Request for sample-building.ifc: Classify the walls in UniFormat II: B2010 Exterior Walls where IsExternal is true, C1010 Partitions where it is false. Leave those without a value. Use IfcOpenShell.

First a look at what the model holds.

```python
import ifcopenshell
import ifcopenshell.util.element

model = ifcopenshell.open("sample-building.ifc")
print(model.schema)
print("classifications:", [c.Name for c in model.by_type("IfcClassification")])
values = [ifcopenshell.util.element.get_pset(e, "Pset_WallCommon", "IsExternal") for e in model.by_type("IfcWall")]
for value in (True, False, None):
    print("IsExternal", value, values.count(value))
```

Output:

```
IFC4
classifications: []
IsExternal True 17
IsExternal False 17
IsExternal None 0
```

```python
import ifcopenshell
import ifcopenshell.api.classification
import ifcopenshell.util.element

model = ifcopenshell.open("sample-building.ifc")

system = ifcopenshell.api.classification.add_classification(model, classification="UniFormat II")

walls = model.by_type("IfcWall")
external = {e: ifcopenshell.util.element.get_pset(e, "Pset_WallCommon", "IsExternal") for e in walls}
for flag, code, name in ((True, "B2010", "Exterior Walls"), (False, "C1010", "Partitions")):
    products = [e for e in walls if external[e] is flag]
    ifcopenshell.api.classification.add_reference(
        model, products=products, classification=system, identification=code, name=name
    )
    print(code, len(products))

model.write("sample-building_rev.ifc")
```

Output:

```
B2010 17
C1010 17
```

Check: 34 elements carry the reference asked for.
